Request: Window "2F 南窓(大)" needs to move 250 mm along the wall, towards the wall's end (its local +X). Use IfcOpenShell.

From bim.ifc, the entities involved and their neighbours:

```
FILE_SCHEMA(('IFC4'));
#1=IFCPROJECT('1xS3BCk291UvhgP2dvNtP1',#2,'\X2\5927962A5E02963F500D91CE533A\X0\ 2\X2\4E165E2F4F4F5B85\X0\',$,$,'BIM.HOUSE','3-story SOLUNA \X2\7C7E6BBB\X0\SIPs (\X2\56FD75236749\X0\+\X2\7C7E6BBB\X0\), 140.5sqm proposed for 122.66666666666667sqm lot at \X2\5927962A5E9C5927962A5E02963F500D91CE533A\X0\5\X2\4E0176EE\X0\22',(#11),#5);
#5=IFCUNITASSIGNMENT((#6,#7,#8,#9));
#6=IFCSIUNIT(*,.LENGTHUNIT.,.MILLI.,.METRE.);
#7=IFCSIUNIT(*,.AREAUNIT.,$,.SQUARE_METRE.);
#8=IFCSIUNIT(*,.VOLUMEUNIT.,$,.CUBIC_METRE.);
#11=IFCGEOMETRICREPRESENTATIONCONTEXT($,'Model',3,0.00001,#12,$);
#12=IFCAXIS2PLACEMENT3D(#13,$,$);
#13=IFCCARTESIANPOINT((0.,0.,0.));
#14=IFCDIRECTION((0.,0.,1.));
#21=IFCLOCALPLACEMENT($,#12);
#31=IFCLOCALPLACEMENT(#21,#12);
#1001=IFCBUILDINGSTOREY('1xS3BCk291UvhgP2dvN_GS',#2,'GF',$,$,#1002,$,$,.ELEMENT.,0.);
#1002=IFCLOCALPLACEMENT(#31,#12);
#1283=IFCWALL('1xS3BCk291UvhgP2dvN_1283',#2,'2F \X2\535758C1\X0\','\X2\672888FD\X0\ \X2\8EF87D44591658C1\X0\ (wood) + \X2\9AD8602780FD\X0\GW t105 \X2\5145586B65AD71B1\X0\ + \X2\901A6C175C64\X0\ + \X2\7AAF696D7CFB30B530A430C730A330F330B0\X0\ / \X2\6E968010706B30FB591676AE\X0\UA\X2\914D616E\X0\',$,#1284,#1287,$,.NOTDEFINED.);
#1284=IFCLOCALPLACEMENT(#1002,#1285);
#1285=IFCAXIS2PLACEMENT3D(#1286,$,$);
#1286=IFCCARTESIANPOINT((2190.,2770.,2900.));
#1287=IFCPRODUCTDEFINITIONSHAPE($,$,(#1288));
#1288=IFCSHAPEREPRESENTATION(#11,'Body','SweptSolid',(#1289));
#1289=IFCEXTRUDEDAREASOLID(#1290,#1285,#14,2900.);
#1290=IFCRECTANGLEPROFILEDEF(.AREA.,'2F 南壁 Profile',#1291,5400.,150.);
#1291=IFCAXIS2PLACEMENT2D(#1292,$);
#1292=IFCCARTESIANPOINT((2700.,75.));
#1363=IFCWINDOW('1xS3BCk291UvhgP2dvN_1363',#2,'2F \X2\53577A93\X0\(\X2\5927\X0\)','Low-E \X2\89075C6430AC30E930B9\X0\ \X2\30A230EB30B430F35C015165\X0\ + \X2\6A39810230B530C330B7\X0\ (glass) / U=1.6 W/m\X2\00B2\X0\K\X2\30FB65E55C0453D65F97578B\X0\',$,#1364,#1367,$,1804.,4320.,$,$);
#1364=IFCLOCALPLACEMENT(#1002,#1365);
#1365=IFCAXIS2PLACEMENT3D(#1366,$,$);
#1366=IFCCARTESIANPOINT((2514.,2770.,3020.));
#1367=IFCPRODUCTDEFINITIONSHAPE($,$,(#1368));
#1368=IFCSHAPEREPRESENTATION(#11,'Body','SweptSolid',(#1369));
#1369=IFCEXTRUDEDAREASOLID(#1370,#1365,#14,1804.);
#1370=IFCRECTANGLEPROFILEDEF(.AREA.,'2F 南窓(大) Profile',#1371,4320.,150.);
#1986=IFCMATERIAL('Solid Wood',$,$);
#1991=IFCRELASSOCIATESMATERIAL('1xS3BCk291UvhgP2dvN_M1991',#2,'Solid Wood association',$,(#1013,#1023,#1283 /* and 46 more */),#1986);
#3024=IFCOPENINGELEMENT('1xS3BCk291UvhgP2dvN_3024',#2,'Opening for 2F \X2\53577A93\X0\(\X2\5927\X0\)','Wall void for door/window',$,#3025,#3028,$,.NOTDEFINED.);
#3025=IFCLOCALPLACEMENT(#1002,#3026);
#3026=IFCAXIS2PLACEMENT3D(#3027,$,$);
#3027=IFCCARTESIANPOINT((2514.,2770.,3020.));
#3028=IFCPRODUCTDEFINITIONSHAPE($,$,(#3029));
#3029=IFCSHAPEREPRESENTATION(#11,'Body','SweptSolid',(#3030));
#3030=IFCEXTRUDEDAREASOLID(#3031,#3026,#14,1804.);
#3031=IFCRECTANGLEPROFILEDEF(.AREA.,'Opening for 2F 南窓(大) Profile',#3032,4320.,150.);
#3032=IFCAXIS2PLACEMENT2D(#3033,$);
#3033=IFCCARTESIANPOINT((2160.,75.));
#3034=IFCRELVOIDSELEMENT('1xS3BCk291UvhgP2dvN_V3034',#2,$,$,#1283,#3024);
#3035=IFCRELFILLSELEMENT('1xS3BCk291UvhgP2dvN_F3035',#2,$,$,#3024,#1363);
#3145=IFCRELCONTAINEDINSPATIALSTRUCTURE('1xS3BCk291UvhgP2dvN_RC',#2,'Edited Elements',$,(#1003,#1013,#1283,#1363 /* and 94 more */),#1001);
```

```python
import ifcopenshell
import ifcopenshell.api.geometry
import ifcopenshell.util.placement
import ifcopenshell.util.unit

model = ifcopenshell.open("bim.ifc")
unit_scale = ifcopenshell.util.unit.calculate_unit_scale(model)

window = model.by_guid("1xS3BCk291UvhgP2dvN_1363")
opening = window.FillsVoids[0].RelatingOpeningElement
wall = opening.VoidsElements[0].RelatingBuildingElement

wall_matrix = ifcopenshell.util.placement.get_local_placement(wall.ObjectPlacement)
shift = wall_matrix[:3, 0] * 0.25 / unit_scale
before = ifcopenshell.util.placement.get_local_placement(window.ObjectPlacement)[:3, 3].copy()

# The window is not placed relative to its opening, so move both.
for product in (opening, window):
    matrix = ifcopenshell.util.placement.get_local_placement(product.ObjectPlacement)
    matrix[:3, 3] += shift
    ifcopenshell.api.geometry.edit_object_placement(model, product=product, matrix=matrix, is_si=False)

after = ifcopenshell.util.placement.get_local_placement(window.ObjectPlacement)[:3, 3]
print("window moved by", (after - before).round(3) + 0.0)

model.write("bim_v2.ifc")
```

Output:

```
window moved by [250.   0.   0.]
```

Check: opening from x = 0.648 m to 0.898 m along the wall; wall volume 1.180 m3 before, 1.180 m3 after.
